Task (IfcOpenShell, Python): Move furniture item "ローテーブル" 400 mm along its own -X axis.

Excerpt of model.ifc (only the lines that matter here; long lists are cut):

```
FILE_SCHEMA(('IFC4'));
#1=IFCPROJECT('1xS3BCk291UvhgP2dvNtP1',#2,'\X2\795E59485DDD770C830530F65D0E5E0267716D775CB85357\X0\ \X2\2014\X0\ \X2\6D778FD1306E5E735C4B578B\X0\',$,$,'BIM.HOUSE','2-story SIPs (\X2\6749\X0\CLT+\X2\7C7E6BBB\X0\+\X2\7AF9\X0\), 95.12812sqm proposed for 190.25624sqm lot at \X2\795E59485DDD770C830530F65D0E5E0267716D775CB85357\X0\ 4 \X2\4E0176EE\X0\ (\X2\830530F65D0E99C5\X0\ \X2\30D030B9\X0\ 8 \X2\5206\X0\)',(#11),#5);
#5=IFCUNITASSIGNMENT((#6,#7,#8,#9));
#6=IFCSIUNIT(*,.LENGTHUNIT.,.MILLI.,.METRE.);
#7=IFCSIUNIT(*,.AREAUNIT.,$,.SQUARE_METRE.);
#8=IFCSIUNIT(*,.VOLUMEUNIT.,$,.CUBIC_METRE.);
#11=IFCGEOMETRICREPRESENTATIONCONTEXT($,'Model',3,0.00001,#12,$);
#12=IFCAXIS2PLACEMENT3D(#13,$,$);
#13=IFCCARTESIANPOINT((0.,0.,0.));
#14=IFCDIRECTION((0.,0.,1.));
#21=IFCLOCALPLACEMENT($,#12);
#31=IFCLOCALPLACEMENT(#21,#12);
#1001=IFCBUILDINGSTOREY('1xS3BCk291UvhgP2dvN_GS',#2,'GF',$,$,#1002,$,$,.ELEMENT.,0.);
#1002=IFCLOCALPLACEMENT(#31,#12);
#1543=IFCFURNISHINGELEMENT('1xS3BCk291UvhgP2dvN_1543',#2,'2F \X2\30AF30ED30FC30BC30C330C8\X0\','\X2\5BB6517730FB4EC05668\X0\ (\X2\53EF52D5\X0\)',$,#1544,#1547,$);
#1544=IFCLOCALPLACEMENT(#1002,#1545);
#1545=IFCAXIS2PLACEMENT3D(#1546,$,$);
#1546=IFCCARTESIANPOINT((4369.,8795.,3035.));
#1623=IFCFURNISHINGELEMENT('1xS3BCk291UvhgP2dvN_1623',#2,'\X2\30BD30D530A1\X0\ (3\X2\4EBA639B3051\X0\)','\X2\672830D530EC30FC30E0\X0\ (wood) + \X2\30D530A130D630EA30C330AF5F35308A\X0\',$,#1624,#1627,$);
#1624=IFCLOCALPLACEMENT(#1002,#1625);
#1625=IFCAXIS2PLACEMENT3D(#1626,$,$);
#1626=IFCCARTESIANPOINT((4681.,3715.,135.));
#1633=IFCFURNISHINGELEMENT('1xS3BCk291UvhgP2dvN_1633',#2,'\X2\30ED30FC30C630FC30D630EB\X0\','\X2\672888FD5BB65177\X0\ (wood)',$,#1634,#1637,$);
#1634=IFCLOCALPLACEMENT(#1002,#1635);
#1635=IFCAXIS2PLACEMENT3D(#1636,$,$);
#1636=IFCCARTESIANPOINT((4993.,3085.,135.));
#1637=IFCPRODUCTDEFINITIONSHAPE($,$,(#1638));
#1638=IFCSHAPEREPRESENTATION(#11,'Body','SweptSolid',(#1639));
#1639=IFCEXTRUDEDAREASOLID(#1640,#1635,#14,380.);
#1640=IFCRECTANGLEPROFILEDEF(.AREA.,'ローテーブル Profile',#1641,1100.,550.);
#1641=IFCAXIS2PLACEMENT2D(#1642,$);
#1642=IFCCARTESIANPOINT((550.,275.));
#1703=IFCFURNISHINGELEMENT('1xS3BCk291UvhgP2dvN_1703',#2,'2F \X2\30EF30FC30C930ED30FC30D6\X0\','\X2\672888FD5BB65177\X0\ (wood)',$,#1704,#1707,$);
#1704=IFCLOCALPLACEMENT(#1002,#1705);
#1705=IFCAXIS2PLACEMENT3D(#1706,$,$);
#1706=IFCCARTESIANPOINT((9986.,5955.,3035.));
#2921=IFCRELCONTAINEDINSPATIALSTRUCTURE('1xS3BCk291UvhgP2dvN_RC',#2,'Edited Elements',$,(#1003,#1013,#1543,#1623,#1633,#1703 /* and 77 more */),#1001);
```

```python
import ifcopenshell
import ifcopenshell.api.geometry
import ifcopenshell.util.placement

model = ifcopenshell.open("model.ifc")

item = model.by_guid("1xS3BCk291UvhgP2dvN_1633")
matrix = ifcopenshell.util.placement.get_local_placement(item.ObjectPlacement)
matrix[:3, 3] -= matrix[:3, 0] * 400.0
ifcopenshell.api.geometry.edit_object_placement(model, product=item, matrix=matrix, is_si=False)

print(ifcopenshell.util.placement.get_local_placement(item.ObjectPlacement).round(3) + 0.0)

model.write("model_edited.ifc")
```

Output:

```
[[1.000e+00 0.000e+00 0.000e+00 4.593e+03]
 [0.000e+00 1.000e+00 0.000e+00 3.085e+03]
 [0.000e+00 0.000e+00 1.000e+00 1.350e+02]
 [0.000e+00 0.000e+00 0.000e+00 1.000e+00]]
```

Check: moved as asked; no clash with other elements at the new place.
